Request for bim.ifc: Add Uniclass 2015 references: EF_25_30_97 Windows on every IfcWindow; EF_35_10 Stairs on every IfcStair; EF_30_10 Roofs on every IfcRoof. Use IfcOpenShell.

First a look at what the model holds.

```python
import ifcopenshell

model = ifcopenshell.open("bim.ifc")
print(model.schema)
print("classifications:", [c.Name for c in model.by_type("IfcClassification")])
for ifc_class in ("IfcDoor", "IfcRoof", "IfcStair", "IfcWall", "IfcWindow"):
    print(ifc_class, len(model.by_type(ifc_class)))
```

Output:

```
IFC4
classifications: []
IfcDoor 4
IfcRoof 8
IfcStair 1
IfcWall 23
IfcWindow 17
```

```python
import ifcopenshell
import ifcopenshell.api.classification

model = ifcopenshell.open("bim.ifc")

system = ifcopenshell.api.classification.add_classification(model, classification="Uniclass 2015")

codes = {
    "IfcWindow": ("EF_25_30_97", "Windows"),
    "IfcStair": ("EF_35_10", "Stairs"),
    "IfcRoof": ("EF_30_10", "Roofs"),
}
for ifc_class, (code, name) in codes.items():
    products = model.by_type(ifc_class)
    ifcopenshell.api.classification.add_reference(
        model, products=products, classification=system, identification=code, name=name
    )
    print(code, len(products))

model.write("bim_rev.ifc")
```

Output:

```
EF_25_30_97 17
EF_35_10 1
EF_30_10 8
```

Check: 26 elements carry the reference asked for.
